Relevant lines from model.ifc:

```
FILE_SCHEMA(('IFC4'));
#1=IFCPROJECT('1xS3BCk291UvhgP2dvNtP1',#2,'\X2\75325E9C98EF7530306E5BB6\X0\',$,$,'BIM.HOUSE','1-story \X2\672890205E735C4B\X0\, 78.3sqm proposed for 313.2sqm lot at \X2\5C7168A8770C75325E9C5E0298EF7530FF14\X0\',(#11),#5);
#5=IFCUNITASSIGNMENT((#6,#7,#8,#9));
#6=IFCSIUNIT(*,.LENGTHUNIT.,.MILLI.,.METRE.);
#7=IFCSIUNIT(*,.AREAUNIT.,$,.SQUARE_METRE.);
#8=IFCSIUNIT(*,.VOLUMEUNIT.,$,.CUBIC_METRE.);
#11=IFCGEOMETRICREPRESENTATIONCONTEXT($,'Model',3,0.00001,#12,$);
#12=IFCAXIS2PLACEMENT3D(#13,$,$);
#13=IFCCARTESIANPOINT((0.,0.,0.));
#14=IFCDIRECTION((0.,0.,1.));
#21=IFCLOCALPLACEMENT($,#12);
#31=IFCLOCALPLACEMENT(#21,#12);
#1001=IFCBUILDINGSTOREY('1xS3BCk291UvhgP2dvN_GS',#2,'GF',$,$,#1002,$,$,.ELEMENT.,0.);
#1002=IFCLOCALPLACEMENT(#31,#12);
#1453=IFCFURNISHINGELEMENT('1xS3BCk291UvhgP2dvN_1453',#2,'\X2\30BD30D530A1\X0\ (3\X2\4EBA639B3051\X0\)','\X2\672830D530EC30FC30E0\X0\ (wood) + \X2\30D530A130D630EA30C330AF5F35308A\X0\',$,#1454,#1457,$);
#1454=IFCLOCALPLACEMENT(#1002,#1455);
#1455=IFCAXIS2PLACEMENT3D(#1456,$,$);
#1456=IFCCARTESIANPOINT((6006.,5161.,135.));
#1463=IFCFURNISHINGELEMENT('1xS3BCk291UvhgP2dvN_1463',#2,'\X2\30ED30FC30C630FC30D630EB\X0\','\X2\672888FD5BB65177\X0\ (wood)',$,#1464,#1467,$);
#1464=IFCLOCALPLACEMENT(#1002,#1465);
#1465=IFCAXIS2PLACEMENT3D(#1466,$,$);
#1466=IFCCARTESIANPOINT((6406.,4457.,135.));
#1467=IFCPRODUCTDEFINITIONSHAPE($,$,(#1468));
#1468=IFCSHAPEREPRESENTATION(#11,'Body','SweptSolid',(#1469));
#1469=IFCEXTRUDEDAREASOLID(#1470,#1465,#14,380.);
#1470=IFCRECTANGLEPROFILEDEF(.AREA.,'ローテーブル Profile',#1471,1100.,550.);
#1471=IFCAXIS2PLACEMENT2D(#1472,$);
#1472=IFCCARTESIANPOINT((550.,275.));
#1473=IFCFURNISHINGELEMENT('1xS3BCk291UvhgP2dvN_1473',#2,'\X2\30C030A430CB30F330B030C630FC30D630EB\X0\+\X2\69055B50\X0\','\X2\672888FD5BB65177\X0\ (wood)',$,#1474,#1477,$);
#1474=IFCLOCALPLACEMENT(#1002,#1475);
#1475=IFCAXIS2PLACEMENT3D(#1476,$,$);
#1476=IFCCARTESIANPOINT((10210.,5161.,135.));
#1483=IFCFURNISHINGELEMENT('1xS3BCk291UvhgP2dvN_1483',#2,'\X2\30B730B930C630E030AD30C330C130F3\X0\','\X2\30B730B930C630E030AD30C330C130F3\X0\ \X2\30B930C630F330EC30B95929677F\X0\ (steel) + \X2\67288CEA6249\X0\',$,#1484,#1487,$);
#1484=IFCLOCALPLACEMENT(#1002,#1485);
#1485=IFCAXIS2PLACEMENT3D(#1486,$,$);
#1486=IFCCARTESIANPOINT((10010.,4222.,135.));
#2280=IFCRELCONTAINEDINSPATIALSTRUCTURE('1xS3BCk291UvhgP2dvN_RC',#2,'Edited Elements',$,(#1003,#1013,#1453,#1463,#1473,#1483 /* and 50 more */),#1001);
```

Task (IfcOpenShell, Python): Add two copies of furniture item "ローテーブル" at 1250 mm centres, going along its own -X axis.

```python
import ifcopenshell
import ifcopenshell.api.geometry
import ifcopenshell.api.root
import ifcopenshell.util.element
import ifcopenshell.util.placement
import ifcopenshell.util.unit

model = ifcopenshell.open("model.ifc")
unit_scale = ifcopenshell.util.unit.calculate_unit_scale(model)


def reuse_history(source, copy):
    """copy_class also copies each property set's owner history, people and application; keep the originals."""
    for rel in copy.IsDefinedBy:
        if rel.is_a("IfcRelDefinesByProperties") and (history := rel.RelatingPropertyDefinition.OwnerHistory):
            rel.RelatingPropertyDefinition.OwnerHistory = source.OwnerHistory
            ifcopenshell.util.element.remove_deep2(model, history)


source = model.by_guid("1xS3BCk291UvhgP2dvN_1463")
base = ifcopenshell.util.placement.get_local_placement(source.ObjectPlacement)
step = -base[:3, 0] * 1.25 / unit_scale

for i in range(1, 3):
    copy = ifcopenshell.api.root.copy_class(model, product=source)
    copy.Representation = ifcopenshell.util.element.copy_deep(
        model, source.Representation, exclude=["IfcGeometricRepresentationContext", "IfcRepresentationMap"]
    )
    reuse_history(source, copy)
    matrix = base.copy()
    matrix[:3, 3] += i * step
    print("added at", matrix[:3, 3].round(3) + 0.0)
    ifcopenshell.api.geometry.edit_object_placement(model, product=copy, matrix=matrix, is_si=False)

model.write("model_rev.ifc")
```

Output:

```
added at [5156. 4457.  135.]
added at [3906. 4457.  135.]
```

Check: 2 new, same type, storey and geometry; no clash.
